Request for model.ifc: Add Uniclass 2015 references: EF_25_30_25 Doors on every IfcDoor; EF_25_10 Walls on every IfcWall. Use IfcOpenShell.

First a look at what the model holds.

```python
import ifcopenshell

model = ifcopenshell.open("model.ifc")
print(model.schema)
print("classifications:", [c.Name for c in model.by_type("IfcClassification")])
for ifc_class in ("IfcDoor", "IfcRoof", "IfcStair", "IfcWall", "IfcWindow"):
    print(ifc_class, len(model.by_type(ifc_class)))
```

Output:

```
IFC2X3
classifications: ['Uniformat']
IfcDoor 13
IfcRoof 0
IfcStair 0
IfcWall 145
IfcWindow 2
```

```python
import ifcopenshell
import ifcopenshell.api.classification

model = ifcopenshell.open("model.ifc")

# IFC2X3 requires Source and Edition and has no link from the project to the system.
system = model.create_entity("IfcClassification", Source="NBS", Edition="2015", Name="Uniclass 2015")

codes = {
    "IfcDoor": ("EF_25_30_25", "Doors"),
    "IfcWall": ("EF_25_10", "Walls"),
}
for ifc_class, (code, name) in codes.items():
    products = model.by_type(ifc_class)
    ifcopenshell.api.classification.add_reference(
        model, products=products, classification=system, identification=code, name=name
    )
    print(code, len(products))

model.write("model_v2.ifc")
```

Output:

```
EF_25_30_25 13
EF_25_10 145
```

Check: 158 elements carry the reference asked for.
